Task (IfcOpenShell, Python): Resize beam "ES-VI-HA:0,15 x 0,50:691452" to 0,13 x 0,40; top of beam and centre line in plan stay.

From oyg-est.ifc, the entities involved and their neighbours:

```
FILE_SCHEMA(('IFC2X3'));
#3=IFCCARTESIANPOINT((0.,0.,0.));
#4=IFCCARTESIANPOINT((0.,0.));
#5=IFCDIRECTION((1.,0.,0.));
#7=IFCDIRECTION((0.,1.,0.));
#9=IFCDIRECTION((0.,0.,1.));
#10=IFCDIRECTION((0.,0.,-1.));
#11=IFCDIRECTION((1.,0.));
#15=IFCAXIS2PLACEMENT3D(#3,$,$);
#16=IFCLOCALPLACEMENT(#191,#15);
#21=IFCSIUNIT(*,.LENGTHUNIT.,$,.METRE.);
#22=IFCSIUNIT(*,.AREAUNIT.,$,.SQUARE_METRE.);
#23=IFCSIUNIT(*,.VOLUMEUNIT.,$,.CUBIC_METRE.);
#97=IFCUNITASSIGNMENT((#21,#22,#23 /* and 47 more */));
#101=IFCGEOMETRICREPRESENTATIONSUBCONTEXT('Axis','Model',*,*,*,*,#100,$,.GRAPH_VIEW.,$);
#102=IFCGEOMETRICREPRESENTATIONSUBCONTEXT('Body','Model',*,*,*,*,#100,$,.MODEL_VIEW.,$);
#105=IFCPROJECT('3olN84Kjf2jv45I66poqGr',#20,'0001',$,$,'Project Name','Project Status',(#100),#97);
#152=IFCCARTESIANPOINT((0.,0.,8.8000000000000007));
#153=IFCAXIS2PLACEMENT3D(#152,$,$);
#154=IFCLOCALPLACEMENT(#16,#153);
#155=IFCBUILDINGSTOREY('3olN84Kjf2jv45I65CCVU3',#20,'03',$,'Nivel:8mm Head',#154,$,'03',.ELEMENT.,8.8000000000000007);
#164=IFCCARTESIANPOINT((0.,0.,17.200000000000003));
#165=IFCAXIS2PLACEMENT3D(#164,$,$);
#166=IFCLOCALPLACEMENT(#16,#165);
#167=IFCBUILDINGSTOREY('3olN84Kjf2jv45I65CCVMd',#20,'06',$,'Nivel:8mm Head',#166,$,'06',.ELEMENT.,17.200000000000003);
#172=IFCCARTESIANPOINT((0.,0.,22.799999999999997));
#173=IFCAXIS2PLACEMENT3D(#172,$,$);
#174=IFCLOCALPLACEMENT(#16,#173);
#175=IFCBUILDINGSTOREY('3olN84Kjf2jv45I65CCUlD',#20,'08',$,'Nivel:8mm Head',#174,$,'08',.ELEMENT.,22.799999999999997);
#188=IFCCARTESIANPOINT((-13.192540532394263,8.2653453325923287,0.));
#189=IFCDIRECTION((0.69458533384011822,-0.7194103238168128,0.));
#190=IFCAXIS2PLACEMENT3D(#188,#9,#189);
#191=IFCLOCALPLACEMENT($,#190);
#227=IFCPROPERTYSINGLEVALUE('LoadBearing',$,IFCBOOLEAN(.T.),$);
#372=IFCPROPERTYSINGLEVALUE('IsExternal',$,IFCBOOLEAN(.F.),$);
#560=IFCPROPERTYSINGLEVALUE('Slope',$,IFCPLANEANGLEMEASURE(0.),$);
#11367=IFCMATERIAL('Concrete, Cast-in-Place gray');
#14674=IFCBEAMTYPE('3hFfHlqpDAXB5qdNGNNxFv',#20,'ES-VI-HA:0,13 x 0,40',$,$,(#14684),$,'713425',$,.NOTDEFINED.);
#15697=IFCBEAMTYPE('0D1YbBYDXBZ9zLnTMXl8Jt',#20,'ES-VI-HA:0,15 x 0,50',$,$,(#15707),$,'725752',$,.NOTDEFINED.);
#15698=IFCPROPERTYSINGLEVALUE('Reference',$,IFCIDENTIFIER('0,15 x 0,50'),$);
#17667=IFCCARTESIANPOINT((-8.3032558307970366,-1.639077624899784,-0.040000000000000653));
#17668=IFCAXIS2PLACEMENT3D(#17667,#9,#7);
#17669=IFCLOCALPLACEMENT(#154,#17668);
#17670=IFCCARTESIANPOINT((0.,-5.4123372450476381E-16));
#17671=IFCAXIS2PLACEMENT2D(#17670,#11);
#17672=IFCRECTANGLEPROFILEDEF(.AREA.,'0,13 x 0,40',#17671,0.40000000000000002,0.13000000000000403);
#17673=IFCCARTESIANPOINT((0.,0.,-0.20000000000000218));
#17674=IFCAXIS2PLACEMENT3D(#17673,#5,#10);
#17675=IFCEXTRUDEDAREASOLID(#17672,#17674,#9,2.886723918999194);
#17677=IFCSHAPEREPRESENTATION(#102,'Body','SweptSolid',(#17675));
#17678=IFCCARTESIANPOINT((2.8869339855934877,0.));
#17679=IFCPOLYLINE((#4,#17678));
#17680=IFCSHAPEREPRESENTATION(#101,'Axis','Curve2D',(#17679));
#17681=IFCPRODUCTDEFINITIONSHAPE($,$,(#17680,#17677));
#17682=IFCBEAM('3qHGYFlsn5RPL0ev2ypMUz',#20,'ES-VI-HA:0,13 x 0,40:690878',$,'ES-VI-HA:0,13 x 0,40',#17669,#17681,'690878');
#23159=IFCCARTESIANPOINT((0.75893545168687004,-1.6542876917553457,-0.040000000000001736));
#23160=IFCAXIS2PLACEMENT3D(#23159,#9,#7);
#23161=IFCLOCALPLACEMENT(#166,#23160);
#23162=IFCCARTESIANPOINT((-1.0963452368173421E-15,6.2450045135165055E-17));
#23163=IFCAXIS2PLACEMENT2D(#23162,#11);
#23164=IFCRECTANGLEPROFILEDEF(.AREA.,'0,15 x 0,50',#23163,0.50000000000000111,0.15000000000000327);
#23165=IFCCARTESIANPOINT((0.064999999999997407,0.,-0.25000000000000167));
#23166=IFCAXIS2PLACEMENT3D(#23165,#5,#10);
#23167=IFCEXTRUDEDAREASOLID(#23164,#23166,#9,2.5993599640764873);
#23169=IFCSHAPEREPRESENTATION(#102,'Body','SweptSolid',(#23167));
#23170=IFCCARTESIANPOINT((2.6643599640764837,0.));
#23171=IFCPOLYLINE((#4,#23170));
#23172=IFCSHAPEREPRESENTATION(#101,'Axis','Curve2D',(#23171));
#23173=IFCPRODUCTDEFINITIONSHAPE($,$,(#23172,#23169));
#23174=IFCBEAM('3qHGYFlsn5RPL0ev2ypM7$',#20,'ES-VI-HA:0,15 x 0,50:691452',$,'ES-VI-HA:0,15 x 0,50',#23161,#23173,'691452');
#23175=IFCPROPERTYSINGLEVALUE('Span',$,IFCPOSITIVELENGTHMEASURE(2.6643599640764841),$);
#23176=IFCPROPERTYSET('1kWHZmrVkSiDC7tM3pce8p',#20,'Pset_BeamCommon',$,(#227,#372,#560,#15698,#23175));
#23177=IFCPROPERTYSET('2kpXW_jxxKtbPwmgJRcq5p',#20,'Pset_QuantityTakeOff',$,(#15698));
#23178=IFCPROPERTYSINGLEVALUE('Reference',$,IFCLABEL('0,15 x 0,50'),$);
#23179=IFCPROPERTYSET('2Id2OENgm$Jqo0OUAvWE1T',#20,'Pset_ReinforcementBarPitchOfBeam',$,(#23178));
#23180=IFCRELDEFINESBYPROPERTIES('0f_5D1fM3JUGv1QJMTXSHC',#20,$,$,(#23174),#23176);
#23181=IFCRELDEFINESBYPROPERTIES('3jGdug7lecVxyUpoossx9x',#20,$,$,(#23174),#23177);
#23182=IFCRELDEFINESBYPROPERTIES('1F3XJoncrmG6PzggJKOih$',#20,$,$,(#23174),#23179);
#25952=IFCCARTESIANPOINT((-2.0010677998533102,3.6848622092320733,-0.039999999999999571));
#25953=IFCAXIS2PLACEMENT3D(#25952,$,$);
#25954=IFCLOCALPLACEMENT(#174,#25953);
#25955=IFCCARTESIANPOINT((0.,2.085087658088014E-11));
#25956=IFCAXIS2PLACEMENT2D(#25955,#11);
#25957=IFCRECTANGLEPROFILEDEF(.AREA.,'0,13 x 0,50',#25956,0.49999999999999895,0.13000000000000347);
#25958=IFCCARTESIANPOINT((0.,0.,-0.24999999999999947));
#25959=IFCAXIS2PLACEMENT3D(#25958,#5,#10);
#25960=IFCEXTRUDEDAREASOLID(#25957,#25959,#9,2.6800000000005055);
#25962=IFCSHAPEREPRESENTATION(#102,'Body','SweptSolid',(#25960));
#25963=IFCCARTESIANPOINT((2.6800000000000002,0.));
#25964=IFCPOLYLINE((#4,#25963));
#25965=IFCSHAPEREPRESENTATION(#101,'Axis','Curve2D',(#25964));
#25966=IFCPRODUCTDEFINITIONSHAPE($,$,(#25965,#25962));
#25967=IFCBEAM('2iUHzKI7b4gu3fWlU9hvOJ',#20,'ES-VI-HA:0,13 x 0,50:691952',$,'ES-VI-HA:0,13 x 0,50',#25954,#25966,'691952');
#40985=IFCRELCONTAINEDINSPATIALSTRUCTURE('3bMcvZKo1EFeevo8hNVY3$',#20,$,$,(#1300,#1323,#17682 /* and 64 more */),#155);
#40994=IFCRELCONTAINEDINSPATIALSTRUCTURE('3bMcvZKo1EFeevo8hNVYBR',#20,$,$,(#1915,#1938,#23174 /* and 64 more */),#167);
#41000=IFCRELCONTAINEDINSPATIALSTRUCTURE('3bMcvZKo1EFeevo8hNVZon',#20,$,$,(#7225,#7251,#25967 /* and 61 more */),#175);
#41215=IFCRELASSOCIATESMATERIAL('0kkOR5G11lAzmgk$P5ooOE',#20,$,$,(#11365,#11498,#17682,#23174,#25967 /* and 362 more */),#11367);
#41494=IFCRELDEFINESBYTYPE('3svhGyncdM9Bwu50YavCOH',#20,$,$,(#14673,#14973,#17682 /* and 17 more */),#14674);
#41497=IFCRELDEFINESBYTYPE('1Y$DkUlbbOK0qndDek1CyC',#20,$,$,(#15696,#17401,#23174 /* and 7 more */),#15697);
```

```python
import ifcopenshell
import ifcopenshell.api.pset
import ifcopenshell.api.type
import ifcopenshell.util.element
import ifcopenshell.util.representation

model = ifcopenshell.open("oyg-est.ifc")

member = model.by_guid("3qHGYFlsn5RPL0ev2ypM7$")
source = next(p for p in model.by_type("IfcRectangleProfileDef") if p.ProfileName == "0,13 x 0,40")

body = ifcopenshell.util.representation.get_representation(member, "Model", "Body")
solid = body.Items[0]
old_profile = solid.SweptArea

# Copy the section's sizes but keep this member's own profile position.
profile = ifcopenshell.util.element.copy(model, source)
# Profiles are centred, so shift by half the change in depth to hold the top.
shift = (old_profile.XDim - profile.XDim) / 2
x, y = old_profile.Position.Location.Coordinates
up = (-1.0, 0.0)  # upwards, in the solid's own plane
location = model.createIfcCartesianPoint((x + up[0] * shift, y + up[1] * shift))
profile.Position = model.createIfcAxis2Placement2D(location, old_profile.Position.RefDirection)
solid.SweptArea = profile
if not model.get_total_inverses(old_profile):
    ifcopenshell.util.element.remove_deep2(model, old_profile)

new_type = model.by_guid("3hFfHlqpDAXB5qdNGNNxFv")
ifcopenshell.api.type.assign_type(
    model, related_objects=[member], relating_type=new_type, should_map_representations=False
)
member.Name = member.Name.replace("0,15 x 0,50", "0,13 x 0,40")
member.ObjectType = "ES-VI-HA:0,13 x 0,40"
pset = model.by_id(ifcopenshell.util.element.get_pset(member, "Pset_BeamCommon", should_inherit=False)["id"])
ifcopenshell.api.pset.edit_pset(model, pset=pset, properties={"Reference": "0,13 x 0,40"})
pset = model.by_id(ifcopenshell.util.element.get_pset(member, "Pset_QuantityTakeOff", should_inherit=False)["id"])
ifcopenshell.api.pset.edit_pset(model, pset=pset, properties={"Reference": "0,13 x 0,40"})
pset = model.by_id(ifcopenshell.util.element.get_pset(member, "Pset_ReinforcementBarPitchOfBeam", should_inherit=False)["id"])
ifcopenshell.api.pset.edit_pset(model, pset=pset, properties={"Reference": "0,13 x 0,40"})

print(solid.SweptArea)

model.write("oyg-est_edited.ifc")
```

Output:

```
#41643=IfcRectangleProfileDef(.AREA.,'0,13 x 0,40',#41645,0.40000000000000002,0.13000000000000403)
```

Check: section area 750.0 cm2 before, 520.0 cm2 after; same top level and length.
